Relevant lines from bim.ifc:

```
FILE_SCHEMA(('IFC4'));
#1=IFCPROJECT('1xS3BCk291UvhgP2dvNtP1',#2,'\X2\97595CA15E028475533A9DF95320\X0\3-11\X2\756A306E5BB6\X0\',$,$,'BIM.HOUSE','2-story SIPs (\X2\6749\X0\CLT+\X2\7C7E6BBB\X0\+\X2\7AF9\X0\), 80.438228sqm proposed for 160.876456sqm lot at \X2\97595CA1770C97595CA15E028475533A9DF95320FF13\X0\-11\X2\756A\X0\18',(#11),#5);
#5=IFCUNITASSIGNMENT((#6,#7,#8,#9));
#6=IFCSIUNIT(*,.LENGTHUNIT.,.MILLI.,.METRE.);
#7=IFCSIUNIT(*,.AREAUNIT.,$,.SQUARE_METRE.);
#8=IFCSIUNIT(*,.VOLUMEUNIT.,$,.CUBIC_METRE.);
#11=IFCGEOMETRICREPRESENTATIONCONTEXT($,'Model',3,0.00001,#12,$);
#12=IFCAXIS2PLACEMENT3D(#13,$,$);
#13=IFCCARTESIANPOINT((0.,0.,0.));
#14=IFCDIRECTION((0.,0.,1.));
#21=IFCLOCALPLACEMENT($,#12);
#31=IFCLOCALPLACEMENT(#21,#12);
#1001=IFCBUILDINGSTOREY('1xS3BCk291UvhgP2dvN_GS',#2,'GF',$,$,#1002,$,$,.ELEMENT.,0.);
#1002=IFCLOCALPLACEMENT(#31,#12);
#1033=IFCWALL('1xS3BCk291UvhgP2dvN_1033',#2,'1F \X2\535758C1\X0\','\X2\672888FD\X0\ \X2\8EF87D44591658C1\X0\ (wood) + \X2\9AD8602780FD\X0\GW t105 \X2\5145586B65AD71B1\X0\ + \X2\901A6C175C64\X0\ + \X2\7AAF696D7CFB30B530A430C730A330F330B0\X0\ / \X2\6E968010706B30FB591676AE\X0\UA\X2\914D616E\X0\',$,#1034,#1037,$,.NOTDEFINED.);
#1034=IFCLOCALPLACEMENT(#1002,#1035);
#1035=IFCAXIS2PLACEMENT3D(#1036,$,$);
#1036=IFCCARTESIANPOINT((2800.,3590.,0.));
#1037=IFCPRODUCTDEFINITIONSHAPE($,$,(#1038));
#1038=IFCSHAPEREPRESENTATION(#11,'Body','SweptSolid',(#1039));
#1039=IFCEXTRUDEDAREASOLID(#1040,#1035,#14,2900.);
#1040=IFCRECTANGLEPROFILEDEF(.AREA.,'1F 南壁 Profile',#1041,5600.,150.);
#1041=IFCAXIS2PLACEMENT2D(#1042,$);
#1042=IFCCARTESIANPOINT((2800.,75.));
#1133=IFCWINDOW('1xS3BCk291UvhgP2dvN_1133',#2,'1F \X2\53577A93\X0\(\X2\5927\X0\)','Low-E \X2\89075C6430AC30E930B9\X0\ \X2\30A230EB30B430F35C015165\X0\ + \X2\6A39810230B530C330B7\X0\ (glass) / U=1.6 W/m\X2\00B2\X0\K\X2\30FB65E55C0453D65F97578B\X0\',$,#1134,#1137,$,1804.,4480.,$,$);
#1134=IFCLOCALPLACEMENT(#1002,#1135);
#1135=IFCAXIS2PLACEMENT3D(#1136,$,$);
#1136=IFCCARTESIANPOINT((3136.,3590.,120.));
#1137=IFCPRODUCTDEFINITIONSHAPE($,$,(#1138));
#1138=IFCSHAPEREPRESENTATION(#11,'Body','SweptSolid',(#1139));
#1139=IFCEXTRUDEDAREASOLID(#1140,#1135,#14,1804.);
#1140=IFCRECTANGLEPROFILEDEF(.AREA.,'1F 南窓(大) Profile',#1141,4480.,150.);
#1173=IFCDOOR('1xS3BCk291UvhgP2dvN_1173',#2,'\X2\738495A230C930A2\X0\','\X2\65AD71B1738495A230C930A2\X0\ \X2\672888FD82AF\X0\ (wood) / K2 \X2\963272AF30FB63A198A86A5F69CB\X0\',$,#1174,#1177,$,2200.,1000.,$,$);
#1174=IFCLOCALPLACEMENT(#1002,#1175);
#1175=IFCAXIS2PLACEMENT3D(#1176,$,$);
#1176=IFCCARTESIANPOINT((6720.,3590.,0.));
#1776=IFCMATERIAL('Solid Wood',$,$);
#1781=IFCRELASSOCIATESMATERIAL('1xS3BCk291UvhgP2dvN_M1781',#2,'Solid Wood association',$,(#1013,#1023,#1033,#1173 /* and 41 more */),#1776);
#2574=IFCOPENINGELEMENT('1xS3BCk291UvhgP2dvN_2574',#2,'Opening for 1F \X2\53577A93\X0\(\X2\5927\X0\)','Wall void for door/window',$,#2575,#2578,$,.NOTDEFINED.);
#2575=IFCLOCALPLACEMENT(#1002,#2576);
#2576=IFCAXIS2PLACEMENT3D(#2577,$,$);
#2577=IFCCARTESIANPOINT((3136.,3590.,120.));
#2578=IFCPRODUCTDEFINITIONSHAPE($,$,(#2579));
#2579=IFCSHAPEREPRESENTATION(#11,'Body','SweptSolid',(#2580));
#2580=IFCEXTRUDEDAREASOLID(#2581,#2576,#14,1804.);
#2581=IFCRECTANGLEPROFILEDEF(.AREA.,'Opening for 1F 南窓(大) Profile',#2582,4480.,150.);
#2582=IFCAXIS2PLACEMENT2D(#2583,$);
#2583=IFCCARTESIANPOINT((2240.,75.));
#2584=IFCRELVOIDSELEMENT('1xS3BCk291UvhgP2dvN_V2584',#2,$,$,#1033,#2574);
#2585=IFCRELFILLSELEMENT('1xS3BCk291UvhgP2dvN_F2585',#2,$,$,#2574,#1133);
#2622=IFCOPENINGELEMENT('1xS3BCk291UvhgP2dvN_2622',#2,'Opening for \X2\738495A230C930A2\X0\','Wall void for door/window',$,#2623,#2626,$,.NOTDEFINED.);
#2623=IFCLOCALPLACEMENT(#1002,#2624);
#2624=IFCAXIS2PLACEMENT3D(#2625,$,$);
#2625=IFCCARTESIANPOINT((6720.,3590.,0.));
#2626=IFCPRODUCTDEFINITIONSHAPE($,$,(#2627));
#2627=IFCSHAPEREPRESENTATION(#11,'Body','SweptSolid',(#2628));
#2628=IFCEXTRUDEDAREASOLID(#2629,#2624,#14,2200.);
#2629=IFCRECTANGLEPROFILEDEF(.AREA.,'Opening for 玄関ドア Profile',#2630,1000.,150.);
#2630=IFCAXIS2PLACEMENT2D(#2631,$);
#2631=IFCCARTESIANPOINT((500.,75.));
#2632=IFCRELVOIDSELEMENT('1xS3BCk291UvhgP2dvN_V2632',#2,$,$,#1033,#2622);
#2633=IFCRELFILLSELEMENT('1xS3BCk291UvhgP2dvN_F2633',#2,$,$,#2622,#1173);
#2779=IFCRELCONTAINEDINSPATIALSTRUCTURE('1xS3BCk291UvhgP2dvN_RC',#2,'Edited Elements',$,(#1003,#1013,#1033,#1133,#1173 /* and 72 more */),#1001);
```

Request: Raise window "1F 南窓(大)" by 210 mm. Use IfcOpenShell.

```python
import numpy as np
import ifcopenshell
import ifcopenshell.api.geometry
import ifcopenshell.util.placement
import ifcopenshell.util.unit

model = ifcopenshell.open("bim.ifc")
unit_scale = ifcopenshell.util.unit.calculate_unit_scale(model)

window = model.by_id(1133)
opening = window.FillsVoids[0].RelatingOpeningElement
dz = 0.21 / unit_scale

shift = np.array([0.0, 0.0, dz])
# The window is not placed relative to its opening, so move both.
for product in (opening, window):
    matrix = ifcopenshell.util.placement.get_local_placement(product.ObjectPlacement)
    matrix[:3, 3] += shift
    ifcopenshell.api.geometry.edit_object_placement(model, product=product, matrix=matrix, is_si=False)

print(f"moved by {dz * unit_scale:+.3f} m")

model.write("bim_v2.ifc")
```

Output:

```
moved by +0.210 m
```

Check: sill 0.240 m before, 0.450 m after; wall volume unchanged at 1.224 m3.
